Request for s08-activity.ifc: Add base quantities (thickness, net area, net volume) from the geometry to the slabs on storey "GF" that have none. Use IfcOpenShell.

First a look at what the model holds.

```python
import ifcopenshell
import ifcopenshell.util.element
import ifcopenshell.util.unit

model = ifcopenshell.open("s08-activity.ifc")
print(model.schema)
for unit_type in ("LENGTHUNIT", "AREAUNIT", "VOLUMEUNIT"):
    print(unit_type, ifcopenshell.util.unit.calculate_unit_scale(model, unit_type))
storey = next(s for s in model.by_type("IfcBuildingStorey") if s.Name == "GF")
slabs = [e for e in ifcopenshell.util.element.get_decomposition(storey) if e.is_a("IfcSlab")]
for e in sorted(slabs, key=lambda e: e.id()):
    print(e.id(), e.is_a(), e.Name, list(ifcopenshell.util.element.get_psets(e, qtos_only=True)), sep=" | ")
```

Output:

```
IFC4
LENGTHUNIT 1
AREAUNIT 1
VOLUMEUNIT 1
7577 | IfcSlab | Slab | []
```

```python
import ifcopenshell
import ifcopenshell.api.pset
import ifcopenshell.geom
import ifcopenshell.util.element
import ifcopenshell.util.shape
import ifcopenshell.util.unit

model = ifcopenshell.open("s08-activity.ifc")
unit_scale = ifcopenshell.util.unit.calculate_unit_scale(model)
area_scale = ifcopenshell.util.unit.calculate_unit_scale(model, "AREAUNIT")
volume_scale = ifcopenshell.util.unit.calculate_unit_scale(model, "VOLUMEUNIT")
settings = ifcopenshell.geom.settings()

storey = next(s for s in model.by_type("IfcBuildingStorey") if s.Name == "GF")
slabs = [e for e in ifcopenshell.util.element.get_decomposition(storey) if e.is_a("IfcSlab")]

for e in sorted(slabs, key=lambda e: e.id()):
    if ifcopenshell.util.element.get_psets(e, qtos_only=True, should_inherit=False):
        continue
    # Geometry comes back in metres, in the element's own axes.
    shape = ifcopenshell.geom.create_shape(settings, e)
    values = {
        "Width": ifcopenshell.util.shape.get_z(shape.geometry) / unit_scale,
        "NetArea": ifcopenshell.util.shape.get_footprint_area(shape.geometry) / area_scale,
        "NetVolume": ifcopenshell.util.shape.get_volume(shape.geometry) / volume_scale,
    }
    qto = ifcopenshell.api.pset.add_qto(model, product=e, name="Qto_SlabBaseQuantities")
    ifcopenshell.api.pset.edit_qto(model, qto=qto, properties=values)
    print(e.id(), {k: round(v, 3) for k, v in values.items()})

model.write("s08-activity_v2.ifc")
```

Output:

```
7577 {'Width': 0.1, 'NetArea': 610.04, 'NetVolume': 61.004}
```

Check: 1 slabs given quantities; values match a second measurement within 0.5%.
